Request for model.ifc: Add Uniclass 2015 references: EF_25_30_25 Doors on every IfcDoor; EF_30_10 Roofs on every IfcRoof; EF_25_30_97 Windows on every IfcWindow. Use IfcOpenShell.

First a look at what the model holds.

```python
import ifcopenshell

model = ifcopenshell.open("model.ifc")
print(model.schema)
print("classifications:", [c.Name for c in model.by_type("IfcClassification")])
for ifc_class in ("IfcDoor", "IfcRoof", "IfcStair", "IfcWall", "IfcWindow"):
    print(ifc_class, len(model.by_type(ifc_class)))
```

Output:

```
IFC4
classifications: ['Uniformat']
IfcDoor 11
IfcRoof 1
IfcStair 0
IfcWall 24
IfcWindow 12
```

```python
import ifcopenshell
import ifcopenshell.api.classification

model = ifcopenshell.open("model.ifc")

system = ifcopenshell.api.classification.add_classification(model, classification="Uniclass 2015")

codes = {
    "IfcDoor": ("EF_25_30_25", "Doors"),
    "IfcRoof": ("EF_30_10", "Roofs"),
    "IfcWindow": ("EF_25_30_97", "Windows"),
}
for ifc_class, (code, name) in codes.items():
    products = model.by_type(ifc_class)
    ifcopenshell.api.classification.add_reference(
        model, products=products, classification=system, identification=code, name=name
    )
    print(code, len(products))

model.write("model_rev.ifc")
```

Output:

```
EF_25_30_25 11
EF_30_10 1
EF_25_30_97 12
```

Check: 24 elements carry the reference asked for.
